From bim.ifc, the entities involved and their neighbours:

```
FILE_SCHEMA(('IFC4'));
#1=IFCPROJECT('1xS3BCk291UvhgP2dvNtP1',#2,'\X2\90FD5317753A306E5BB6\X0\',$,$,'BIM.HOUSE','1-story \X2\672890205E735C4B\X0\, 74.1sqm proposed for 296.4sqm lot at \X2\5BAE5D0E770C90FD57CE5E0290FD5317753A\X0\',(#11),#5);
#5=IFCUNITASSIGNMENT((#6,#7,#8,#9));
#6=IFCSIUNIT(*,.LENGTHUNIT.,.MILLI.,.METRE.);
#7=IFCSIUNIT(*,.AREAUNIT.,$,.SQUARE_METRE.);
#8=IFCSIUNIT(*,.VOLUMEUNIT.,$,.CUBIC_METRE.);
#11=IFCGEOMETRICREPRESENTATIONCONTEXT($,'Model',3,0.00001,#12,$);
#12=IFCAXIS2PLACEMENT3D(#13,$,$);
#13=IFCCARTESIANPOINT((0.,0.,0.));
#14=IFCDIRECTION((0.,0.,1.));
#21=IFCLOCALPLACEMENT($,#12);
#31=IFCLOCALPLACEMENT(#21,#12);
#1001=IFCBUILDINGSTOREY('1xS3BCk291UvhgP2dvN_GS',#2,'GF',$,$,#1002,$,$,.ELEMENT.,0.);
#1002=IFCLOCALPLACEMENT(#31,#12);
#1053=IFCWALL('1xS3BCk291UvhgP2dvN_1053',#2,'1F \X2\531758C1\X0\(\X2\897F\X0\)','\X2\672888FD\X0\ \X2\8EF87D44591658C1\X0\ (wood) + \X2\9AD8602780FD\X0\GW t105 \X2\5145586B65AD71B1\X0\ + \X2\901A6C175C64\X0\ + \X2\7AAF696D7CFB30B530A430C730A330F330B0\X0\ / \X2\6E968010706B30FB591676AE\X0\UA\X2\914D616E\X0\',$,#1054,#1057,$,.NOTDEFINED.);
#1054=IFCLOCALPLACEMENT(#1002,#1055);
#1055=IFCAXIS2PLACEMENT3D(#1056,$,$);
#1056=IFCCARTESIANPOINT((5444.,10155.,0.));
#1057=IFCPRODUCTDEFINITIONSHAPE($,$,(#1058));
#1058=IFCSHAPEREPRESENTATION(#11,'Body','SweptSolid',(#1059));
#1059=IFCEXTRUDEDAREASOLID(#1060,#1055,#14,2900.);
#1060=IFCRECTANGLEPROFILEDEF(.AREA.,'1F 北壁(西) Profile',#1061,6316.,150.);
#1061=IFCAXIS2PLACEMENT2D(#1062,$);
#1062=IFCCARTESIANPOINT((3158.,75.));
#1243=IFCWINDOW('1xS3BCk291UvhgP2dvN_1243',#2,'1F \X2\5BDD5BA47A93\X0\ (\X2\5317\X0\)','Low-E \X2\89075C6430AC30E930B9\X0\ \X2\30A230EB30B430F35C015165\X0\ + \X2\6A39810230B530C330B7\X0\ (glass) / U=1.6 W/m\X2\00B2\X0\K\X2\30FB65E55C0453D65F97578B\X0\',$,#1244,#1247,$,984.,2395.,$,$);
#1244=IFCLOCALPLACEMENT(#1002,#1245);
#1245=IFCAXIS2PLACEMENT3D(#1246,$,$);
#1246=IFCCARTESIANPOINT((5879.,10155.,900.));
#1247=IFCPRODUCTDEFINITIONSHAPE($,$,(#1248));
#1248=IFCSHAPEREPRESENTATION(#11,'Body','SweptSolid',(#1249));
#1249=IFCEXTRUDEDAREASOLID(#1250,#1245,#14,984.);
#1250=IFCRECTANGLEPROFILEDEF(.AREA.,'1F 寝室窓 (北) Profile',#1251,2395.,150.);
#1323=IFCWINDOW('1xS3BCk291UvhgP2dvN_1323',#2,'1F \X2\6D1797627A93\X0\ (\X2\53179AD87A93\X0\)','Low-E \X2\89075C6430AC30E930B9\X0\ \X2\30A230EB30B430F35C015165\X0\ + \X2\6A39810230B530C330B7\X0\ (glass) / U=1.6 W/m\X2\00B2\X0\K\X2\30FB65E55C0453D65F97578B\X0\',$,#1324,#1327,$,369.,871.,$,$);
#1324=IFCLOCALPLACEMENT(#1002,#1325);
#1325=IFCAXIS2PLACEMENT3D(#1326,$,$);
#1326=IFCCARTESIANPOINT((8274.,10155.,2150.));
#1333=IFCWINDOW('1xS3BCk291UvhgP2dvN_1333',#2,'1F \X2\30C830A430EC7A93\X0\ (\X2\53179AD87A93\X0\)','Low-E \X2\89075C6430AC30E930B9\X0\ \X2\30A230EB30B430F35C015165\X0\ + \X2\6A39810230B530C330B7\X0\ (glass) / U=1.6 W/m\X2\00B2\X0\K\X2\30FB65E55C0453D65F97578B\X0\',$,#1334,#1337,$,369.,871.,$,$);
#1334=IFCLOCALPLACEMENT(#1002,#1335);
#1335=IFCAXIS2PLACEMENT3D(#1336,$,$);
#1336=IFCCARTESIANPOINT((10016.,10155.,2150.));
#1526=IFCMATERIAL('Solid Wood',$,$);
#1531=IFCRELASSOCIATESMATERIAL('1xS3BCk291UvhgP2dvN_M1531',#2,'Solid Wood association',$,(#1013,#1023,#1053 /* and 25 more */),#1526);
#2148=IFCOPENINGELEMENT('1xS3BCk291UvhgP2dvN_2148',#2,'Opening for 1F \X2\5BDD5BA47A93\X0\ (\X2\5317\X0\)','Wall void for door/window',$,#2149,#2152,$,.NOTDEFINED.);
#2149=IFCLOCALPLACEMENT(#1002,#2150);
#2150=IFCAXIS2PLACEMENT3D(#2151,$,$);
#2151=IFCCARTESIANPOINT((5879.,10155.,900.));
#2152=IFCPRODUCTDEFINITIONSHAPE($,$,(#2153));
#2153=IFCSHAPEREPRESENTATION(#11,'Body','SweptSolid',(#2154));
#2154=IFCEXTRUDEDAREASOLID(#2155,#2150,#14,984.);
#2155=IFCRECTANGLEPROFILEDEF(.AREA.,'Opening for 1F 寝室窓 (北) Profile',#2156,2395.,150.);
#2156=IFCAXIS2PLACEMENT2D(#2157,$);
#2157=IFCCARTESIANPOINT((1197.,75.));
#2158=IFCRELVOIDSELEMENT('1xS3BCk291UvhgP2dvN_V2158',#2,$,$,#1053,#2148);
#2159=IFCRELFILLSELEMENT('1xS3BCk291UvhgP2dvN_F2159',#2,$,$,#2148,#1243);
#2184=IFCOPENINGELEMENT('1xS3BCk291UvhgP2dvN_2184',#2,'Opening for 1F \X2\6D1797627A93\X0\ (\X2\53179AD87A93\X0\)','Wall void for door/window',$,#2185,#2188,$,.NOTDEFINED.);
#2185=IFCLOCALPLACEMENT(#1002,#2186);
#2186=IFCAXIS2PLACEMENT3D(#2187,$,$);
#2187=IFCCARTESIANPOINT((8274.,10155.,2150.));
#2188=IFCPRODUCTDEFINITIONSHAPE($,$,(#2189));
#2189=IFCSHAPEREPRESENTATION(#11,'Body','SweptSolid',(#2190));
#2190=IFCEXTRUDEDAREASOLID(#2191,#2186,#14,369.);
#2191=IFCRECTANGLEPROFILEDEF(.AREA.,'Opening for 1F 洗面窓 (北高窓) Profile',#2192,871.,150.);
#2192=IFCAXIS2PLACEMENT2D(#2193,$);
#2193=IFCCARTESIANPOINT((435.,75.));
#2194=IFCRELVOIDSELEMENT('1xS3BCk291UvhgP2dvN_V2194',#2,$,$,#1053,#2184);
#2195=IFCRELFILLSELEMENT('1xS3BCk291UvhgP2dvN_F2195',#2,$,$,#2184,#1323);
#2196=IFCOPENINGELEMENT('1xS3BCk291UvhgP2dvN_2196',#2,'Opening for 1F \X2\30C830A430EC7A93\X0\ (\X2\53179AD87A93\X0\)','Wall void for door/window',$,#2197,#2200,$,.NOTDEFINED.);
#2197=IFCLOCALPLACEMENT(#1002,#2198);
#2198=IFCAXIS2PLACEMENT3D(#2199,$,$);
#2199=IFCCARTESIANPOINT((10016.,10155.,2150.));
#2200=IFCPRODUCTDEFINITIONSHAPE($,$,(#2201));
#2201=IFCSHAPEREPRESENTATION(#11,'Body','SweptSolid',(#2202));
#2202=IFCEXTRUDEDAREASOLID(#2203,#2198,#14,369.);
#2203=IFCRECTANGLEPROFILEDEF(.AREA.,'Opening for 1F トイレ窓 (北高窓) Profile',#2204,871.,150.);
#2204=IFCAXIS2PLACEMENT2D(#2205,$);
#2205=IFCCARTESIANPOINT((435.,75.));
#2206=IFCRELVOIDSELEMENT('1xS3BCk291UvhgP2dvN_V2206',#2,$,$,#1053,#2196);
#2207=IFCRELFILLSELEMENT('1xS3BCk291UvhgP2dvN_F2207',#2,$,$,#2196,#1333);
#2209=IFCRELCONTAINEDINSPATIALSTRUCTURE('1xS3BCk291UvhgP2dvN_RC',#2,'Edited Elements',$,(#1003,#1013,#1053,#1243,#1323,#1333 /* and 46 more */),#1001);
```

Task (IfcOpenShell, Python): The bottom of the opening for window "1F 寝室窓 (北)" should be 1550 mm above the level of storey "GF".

```python
import numpy as np
import ifcopenshell
import ifcopenshell.api.geometry
import ifcopenshell.geom
import ifcopenshell.util.element
import ifcopenshell.util.placement
import ifcopenshell.util.shape
import ifcopenshell.util.unit

model = ifcopenshell.open("bim.ifc")
unit_scale = ifcopenshell.util.unit.calculate_unit_scale(model)

window = model.by_guid("1xS3BCk291UvhgP2dvN_1243")
opening = window.FillsVoids[0].RelatingOpeningElement
storey = ifcopenshell.util.element.get_container(window, ifc_class="IfcBuildingStorey")
level = ifcopenshell.util.placement.get_local_placement(storey.ObjectPlacement)[2, 3]

# The opening's origin need not be at the sill, so measure its lowest point.
shape = ifcopenshell.geom.create_shape(ifcopenshell.geom.settings(), opening)
bottom = ifcopenshell.util.shape.get_shape_bottom_elevation(shape, shape.geometry) / unit_scale
dz = level + 1.55 / unit_scale - bottom

shift = np.array([0.0, 0.0, dz])
# The window is not placed relative to its opening, so move both.
for product in (opening, window):
    matrix = ifcopenshell.util.placement.get_local_placement(product.ObjectPlacement)
    matrix[:3, 3] += shift
    ifcopenshell.api.geometry.edit_object_placement(model, product=product, matrix=matrix, is_si=False)

print(f"moved by {dz * unit_scale:+.3f} m")

model.write("bim-out.ifc")
```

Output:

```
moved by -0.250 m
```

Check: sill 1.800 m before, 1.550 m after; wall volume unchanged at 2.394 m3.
